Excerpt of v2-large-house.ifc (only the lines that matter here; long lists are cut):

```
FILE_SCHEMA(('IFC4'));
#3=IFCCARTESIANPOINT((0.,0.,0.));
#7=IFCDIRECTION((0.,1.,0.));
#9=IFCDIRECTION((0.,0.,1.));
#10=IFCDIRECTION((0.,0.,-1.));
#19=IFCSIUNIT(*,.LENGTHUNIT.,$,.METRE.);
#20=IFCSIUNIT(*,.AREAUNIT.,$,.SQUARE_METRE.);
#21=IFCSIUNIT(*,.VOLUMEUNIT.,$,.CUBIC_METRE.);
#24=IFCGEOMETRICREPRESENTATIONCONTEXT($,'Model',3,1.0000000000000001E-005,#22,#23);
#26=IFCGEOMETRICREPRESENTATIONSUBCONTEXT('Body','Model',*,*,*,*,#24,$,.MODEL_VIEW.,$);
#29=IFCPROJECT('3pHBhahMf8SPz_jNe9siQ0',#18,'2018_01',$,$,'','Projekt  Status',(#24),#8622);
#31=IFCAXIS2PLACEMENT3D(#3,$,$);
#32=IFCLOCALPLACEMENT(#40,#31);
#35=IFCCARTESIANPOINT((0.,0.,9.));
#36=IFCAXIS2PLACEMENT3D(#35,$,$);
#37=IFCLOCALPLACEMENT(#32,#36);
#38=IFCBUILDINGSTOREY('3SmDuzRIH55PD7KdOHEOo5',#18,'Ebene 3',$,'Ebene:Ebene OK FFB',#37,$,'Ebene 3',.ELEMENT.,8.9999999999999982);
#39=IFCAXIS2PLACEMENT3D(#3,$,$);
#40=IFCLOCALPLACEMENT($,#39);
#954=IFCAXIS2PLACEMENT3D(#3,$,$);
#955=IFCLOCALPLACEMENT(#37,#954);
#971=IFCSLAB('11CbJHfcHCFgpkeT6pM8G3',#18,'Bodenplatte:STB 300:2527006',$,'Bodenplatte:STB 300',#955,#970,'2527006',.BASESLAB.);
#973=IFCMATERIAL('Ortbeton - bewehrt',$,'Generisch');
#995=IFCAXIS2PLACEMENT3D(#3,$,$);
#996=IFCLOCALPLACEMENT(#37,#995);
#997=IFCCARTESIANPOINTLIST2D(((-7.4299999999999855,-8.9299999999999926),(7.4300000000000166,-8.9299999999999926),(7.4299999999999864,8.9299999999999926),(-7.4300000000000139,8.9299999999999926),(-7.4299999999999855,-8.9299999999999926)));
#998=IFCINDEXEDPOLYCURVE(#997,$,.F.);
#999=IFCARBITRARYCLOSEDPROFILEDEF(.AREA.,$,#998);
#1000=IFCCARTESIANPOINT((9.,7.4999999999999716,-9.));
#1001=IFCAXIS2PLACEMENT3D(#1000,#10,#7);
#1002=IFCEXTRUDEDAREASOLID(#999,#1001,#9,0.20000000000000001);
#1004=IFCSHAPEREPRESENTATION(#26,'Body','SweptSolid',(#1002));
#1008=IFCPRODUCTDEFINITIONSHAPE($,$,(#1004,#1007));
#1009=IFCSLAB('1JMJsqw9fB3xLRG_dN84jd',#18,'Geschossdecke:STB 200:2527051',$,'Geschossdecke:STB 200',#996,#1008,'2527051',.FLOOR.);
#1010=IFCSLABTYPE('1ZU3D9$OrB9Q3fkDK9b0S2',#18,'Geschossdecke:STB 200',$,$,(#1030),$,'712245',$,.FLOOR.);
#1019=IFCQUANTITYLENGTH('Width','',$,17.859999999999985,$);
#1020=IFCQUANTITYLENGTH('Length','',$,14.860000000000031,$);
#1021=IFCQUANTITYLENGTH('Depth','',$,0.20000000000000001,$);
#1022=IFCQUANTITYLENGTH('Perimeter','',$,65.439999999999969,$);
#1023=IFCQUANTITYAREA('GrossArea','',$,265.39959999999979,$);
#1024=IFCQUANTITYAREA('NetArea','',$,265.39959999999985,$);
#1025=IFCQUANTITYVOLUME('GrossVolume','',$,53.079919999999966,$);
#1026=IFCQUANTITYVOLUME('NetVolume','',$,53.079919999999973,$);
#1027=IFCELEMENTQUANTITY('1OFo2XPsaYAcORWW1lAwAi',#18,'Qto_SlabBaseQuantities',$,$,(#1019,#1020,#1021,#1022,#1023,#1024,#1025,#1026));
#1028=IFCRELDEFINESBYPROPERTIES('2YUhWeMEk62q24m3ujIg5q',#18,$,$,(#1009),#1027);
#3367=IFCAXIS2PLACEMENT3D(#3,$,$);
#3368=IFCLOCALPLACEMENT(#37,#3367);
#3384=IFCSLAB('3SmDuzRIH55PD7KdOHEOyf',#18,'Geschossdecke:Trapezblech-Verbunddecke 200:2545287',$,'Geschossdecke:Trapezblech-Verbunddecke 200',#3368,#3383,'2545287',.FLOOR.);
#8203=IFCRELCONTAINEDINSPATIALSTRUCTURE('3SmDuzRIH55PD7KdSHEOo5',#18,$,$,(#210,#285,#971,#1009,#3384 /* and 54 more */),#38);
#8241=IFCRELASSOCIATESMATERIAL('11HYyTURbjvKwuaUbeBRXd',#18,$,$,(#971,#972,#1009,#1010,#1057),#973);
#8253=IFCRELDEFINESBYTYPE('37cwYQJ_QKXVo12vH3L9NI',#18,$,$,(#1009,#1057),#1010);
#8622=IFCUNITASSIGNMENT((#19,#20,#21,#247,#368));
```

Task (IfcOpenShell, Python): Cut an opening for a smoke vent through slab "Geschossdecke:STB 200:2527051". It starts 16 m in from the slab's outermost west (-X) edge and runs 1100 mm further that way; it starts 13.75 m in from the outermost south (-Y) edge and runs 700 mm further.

```python
import numpy as np
import ifcopenshell
import ifcopenshell.api.feature
import ifcopenshell.api.geometry
import ifcopenshell.api.pset
import ifcopenshell.api.root
import ifcopenshell.geom
import ifcopenshell.util.element
import ifcopenshell.util.placement
import ifcopenshell.util.representation
import ifcopenshell.util.shape
import ifcopenshell.util.unit

model = ifcopenshell.open("v2-large-house.ifc")
unit_scale = ifcopenshell.util.unit.calculate_unit_scale(model)
area_scale = ifcopenshell.util.unit.calculate_unit_scale(model, "AREAUNIT")
volume_scale = ifcopenshell.util.unit.calculate_unit_scale(model, "VOLUMEUNIT")
settings = ifcopenshell.geom.settings()


def volume(element):
    """Net volume in cubic metres, openings subtracted."""
    shape = ifcopenshell.geom.create_shape(settings, element)
    return ifcopenshell.util.shape.get_volume(shape.geometry)


slab = model.by_guid("1JMJsqw9fB3xLRG_dN84jd")
before = volume(slab)

# Extent in the slab's own axes, in metres. The edges named are its -X and -Y sides.
slab_shape = ifcopenshell.geom.create_shape(settings, slab)
vertices = ifcopenshell.util.shape.get_vertices(slab_shape.geometry)
x_min, y_min, bottom = vertices.min(axis=0)
top = vertices[:, 2].max()

opening = ifcopenshell.api.root.create_entity(model, ifc_class="IfcOpeningElement", name="Smoke vent opening", predefined_type="OPENING")
context = ifcopenshell.util.representation.get_context(model, "Model", "Body", "MODEL_VIEW")
width, depth = 1.1, 0.7
outline = [(0.0, 0.0), (width, 0.0), (width, depth), (0.0, depth), (0.0, 0.0)]
# Overshoot both faces by 50 mm so the cut is clean.
shape = ifcopenshell.api.geometry.add_slab_representation(
    model, context=context, depth=top - bottom + 0.1, polyline=outline
)
ifcopenshell.api.geometry.assign_representation(model, product=opening, representation=shape)

matrix = ifcopenshell.util.placement.get_local_placement(slab.ObjectPlacement)
matrix[:, 3] = matrix @ np.append(np.array([x_min + 16, y_min + 13.75, bottom - 0.05]) / unit_scale, 1.0)
ifcopenshell.api.geometry.edit_object_placement(model, product=opening, matrix=matrix, is_si=False)
ifcopenshell.api.feature.add_feature(model, feature=opening, element=slab)

after = volume(slab)

# Update the slab's stored quantities.
qto = model.by_id(ifcopenshell.util.element.get_pset(slab, "Qto_SlabBaseQuantities", should_inherit=False)["id"])
ifcopenshell.api.pset.edit_qto(model, qto=qto, properties={
    "NetArea": after / (top - bottom) / area_scale,
    "NetVolume": after / volume_scale,
})

print(f"slab volume {before:.3f} -> {after:.3f} m3")

model.write("v2-large-house_updated.ifc")
```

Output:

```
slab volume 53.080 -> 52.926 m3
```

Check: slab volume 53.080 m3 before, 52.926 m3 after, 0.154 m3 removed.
